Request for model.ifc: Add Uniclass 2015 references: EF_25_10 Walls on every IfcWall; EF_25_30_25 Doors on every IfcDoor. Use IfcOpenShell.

First a look at what the model holds.

```python
import ifcopenshell

model = ifcopenshell.open("model.ifc")
print(model.schema)
print("classifications:", [c.Name for c in model.by_type("IfcClassification")])
for ifc_class in ("IfcDoor", "IfcRoof", "IfcStair", "IfcWall", "IfcWindow"):
    print(ifc_class, len(model.by_type(ifc_class)))
```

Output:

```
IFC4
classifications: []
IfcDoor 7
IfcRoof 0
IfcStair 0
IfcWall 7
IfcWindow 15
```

```python
import ifcopenshell
import ifcopenshell.api.classification

model = ifcopenshell.open("model.ifc")

system = ifcopenshell.api.classification.add_classification(model, classification="Uniclass 2015")

codes = {
    "IfcWall": ("EF_25_10", "Walls"),
    "IfcDoor": ("EF_25_30_25", "Doors"),
}
for ifc_class, (code, name) in codes.items():
    products = model.by_type(ifc_class)
    ifcopenshell.api.classification.add_reference(
        model, products=products, classification=system, identification=code, name=name
    )
    print(code, len(products))

model.write("model_updated.ifc")
```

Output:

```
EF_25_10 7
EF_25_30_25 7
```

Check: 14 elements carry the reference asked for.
